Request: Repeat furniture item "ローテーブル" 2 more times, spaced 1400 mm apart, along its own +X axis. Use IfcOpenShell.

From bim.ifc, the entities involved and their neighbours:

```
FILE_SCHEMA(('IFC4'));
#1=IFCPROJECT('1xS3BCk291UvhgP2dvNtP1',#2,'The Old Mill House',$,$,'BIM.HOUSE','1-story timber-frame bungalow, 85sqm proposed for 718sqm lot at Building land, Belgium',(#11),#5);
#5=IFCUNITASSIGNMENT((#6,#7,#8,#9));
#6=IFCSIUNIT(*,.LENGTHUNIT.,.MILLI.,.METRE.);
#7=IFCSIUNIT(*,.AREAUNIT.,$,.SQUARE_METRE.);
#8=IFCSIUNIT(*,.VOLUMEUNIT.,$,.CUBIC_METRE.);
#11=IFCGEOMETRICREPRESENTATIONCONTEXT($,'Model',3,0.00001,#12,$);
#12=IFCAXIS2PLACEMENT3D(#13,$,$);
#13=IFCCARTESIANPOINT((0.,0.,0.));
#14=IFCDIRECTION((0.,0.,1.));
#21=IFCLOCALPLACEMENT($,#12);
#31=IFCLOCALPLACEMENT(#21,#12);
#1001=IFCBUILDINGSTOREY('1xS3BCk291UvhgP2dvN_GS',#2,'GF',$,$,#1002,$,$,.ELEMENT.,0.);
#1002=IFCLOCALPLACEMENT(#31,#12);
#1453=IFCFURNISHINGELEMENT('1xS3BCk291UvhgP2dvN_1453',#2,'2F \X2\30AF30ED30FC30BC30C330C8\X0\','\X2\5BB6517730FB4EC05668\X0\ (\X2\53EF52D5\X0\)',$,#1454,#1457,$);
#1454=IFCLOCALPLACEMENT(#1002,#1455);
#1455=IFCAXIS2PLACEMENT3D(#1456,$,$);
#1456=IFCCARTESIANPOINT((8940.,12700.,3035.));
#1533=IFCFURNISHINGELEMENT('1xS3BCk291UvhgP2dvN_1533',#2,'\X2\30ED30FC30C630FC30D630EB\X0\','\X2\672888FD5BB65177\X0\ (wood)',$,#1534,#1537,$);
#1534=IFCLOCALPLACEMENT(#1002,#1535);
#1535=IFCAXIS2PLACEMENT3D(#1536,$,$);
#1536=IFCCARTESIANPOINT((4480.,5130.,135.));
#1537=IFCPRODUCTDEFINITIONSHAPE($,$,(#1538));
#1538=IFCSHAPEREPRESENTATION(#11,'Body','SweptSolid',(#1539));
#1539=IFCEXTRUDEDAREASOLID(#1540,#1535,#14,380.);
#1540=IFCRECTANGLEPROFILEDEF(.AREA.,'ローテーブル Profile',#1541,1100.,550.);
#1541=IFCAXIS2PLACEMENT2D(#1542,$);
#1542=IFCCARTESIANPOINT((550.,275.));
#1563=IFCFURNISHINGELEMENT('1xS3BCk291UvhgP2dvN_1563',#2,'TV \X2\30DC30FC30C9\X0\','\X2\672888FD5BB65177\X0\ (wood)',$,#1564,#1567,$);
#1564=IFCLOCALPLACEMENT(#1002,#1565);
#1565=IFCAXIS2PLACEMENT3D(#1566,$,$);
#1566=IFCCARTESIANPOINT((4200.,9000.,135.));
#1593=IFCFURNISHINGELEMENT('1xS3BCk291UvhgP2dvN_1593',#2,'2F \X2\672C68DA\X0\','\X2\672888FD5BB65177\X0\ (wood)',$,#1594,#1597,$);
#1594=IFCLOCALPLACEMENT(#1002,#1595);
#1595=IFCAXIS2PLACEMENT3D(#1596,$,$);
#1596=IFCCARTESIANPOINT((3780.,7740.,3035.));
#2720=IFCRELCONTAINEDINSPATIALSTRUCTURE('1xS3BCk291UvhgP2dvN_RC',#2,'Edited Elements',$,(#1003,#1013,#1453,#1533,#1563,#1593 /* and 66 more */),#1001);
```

```python
import ifcopenshell
import ifcopenshell.api.geometry
import ifcopenshell.api.root
import ifcopenshell.util.element
import ifcopenshell.util.placement
import ifcopenshell.util.unit

model = ifcopenshell.open("bim.ifc")
unit_scale = ifcopenshell.util.unit.calculate_unit_scale(model)


def reuse_history(source, copy):
    """copy_class also copies each property set's owner history, people and application; keep the originals."""
    for rel in copy.IsDefinedBy:
        if rel.is_a("IfcRelDefinesByProperties") and (history := rel.RelatingPropertyDefinition.OwnerHistory):
            rel.RelatingPropertyDefinition.OwnerHistory = source.OwnerHistory
            ifcopenshell.util.element.remove_deep2(model, history)


source = model.by_id(1533)
base = ifcopenshell.util.placement.get_local_placement(source.ObjectPlacement)
step = base[:3, 0] * 1.4 / unit_scale

for i in range(1, 3):
    copy = ifcopenshell.api.root.copy_class(model, product=source)
    copy.Representation = ifcopenshell.util.element.copy_deep(
        model, source.Representation, exclude=["IfcGeometricRepresentationContext", "IfcRepresentationMap"]
    )
    reuse_history(source, copy)
    matrix = base.copy()
    matrix[:3, 3] += i * step
    print("added at", matrix[:3, 3].round(3) + 0.0)
    ifcopenshell.api.geometry.edit_object_placement(model, product=copy, matrix=matrix, is_si=False)

model.write("bim_v2.ifc")
```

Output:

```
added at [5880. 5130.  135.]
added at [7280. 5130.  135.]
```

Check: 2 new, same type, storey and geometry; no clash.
